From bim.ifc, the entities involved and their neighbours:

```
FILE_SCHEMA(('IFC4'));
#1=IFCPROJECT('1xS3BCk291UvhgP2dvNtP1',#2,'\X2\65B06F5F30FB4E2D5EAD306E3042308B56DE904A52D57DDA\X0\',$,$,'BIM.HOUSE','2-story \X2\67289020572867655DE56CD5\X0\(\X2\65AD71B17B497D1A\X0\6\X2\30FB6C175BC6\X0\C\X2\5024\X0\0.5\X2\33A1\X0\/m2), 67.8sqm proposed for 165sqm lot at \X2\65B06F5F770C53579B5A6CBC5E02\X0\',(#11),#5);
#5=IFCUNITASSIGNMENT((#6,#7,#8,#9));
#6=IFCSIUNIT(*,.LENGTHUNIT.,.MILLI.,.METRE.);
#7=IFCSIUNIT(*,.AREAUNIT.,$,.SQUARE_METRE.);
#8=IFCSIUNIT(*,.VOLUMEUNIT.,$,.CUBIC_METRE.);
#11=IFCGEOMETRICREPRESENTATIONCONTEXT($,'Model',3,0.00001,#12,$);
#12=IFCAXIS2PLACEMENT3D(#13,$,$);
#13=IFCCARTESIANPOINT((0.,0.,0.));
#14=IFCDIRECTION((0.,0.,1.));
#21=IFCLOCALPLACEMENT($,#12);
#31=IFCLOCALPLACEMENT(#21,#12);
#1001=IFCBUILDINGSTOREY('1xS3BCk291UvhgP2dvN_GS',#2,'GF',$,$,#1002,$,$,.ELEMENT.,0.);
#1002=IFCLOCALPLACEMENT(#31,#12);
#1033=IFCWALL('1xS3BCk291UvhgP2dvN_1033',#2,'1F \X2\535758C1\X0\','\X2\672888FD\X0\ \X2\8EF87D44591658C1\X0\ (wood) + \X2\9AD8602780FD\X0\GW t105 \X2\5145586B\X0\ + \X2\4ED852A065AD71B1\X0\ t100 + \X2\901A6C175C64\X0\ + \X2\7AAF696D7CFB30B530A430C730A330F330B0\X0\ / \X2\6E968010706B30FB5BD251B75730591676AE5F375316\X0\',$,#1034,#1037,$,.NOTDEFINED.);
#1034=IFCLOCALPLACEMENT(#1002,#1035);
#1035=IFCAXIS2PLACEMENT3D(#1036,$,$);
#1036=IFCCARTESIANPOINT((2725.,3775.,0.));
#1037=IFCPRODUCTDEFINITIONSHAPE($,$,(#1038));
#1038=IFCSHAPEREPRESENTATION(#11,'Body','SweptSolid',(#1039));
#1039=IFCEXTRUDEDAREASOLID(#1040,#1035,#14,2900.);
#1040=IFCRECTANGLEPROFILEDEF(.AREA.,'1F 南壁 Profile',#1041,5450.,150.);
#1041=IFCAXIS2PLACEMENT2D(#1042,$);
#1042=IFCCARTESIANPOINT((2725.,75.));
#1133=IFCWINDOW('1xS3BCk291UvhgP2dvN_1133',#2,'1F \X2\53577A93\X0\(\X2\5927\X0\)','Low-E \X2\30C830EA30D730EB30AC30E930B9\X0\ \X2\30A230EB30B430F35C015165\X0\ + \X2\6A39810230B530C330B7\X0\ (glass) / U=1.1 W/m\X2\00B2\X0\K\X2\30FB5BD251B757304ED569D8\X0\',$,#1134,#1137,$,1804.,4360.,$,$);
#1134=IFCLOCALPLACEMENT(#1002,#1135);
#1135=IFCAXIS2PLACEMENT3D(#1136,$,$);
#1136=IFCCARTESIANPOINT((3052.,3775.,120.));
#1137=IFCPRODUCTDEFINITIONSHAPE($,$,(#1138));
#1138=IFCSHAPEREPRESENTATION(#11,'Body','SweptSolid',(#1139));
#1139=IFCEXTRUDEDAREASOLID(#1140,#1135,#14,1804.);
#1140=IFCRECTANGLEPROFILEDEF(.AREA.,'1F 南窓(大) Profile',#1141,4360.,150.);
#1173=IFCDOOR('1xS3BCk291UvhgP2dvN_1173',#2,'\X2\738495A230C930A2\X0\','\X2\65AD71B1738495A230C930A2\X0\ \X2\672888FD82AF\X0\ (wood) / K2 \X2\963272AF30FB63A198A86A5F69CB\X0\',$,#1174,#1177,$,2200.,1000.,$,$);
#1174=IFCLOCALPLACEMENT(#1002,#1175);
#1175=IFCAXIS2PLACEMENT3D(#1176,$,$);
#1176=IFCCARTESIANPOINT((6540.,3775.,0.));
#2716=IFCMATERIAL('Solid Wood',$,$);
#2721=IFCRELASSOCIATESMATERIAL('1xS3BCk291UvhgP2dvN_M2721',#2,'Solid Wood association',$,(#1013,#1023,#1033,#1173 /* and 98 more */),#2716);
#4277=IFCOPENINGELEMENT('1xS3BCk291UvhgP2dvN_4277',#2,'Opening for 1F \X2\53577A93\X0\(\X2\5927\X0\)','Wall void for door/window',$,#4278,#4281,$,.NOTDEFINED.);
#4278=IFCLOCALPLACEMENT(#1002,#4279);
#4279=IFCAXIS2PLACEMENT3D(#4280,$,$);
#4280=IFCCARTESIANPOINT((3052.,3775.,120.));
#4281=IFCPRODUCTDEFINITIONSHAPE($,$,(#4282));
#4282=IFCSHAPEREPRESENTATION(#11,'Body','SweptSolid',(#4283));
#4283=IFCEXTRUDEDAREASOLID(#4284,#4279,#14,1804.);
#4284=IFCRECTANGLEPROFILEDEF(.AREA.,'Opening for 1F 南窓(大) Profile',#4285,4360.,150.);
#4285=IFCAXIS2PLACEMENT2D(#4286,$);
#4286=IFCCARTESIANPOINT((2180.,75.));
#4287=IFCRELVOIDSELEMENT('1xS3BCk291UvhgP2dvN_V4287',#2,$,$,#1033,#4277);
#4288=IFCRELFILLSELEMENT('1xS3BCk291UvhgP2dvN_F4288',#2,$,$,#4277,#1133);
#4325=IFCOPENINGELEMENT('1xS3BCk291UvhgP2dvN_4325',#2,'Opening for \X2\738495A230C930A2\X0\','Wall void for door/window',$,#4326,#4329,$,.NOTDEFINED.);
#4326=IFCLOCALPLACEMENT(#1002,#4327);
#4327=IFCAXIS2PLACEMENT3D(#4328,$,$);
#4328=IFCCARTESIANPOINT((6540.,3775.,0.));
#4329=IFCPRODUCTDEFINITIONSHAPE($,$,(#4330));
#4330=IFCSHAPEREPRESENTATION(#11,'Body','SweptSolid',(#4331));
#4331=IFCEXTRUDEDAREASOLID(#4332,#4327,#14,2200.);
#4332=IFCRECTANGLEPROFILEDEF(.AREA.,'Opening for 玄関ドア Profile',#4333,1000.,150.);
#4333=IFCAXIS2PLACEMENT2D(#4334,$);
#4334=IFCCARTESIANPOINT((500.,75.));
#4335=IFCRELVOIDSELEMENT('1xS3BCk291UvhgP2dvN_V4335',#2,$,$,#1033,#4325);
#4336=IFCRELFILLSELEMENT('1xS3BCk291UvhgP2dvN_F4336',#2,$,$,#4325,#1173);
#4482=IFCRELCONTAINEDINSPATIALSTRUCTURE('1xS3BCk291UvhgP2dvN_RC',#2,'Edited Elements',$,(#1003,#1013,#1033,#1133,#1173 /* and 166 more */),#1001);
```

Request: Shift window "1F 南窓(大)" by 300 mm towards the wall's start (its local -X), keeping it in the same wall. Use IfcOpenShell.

```python
import ifcopenshell
import ifcopenshell.api.geometry
import ifcopenshell.util.placement

model = ifcopenshell.open("bim.ifc")

window = model.by_guid("1xS3BCk291UvhgP2dvN_1133")
opening = window.FillsVoids[0].RelatingOpeningElement
wall = opening.VoidsElements[0].RelatingBuildingElement

wall_matrix = ifcopenshell.util.placement.get_local_placement(wall.ObjectPlacement)
shift = wall_matrix[:3, 0] * -300.0
before = ifcopenshell.util.placement.get_local_placement(window.ObjectPlacement)[:3, 3].copy()

# The window is not placed relative to its opening, so move both.
for product in (opening, window):
    matrix = ifcopenshell.util.placement.get_local_placement(product.ObjectPlacement)
    matrix[:3, 3] += shift
    ifcopenshell.api.geometry.edit_object_placement(model, product=product, matrix=matrix, is_si=False)

after = ifcopenshell.util.placement.get_local_placement(window.ObjectPlacement)[:3, 3]
print("window moved by", (after - before).round(3) + 0.0)

model.write("bim_v2.ifc")
```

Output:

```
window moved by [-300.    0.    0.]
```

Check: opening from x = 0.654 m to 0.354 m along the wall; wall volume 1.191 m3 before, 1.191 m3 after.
